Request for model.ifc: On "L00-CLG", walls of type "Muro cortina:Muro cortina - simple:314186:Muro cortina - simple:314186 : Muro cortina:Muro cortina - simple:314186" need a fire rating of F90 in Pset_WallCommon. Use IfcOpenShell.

First a look at what the model holds.

```python
import ifcopenshell
import ifcopenshell.util.element

model = ifcopenshell.open("model.ifc")
print(model.schema)
storey = next(s for s in model.by_type("IfcBuildingStorey") if s.Name == "L00-CLG")
walls = [e for e in ifcopenshell.util.element.get_decomposition(storey) if e.is_a("IfcWall")]
seen = {}
for e in walls:
    element_type = ifcopenshell.util.element.get_type(e)
    key = (element_type.Name if element_type != e and element_type else None, ifcopenshell.util.element.get_pset(e, "Pset_WallCommon", "FireRating"))
    seen[key] = seen.get(key, 0) + 1
for (name, value), count in sorted(seen.items(), key=str):
    print(count, "x", name, "|", value)
```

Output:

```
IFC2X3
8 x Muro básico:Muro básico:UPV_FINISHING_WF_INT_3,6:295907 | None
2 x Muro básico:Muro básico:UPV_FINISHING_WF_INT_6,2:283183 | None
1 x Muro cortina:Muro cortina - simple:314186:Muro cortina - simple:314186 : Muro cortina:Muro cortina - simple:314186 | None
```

```python
import ifcopenshell
import ifcopenshell.api.pset
import ifcopenshell.util.element

model = ifcopenshell.open("model.ifc")

storey = next(s for s in model.by_type("IfcBuildingStorey") if s.Name == "L00-CLG")
walls = [e for e in ifcopenshell.util.element.get_decomposition(storey) if e.is_a("IfcWall")]

count = 0
for e in walls:
    element_type = ifcopenshell.util.element.get_type(e)
    if element_type in (None, e) or element_type.Name != "Muro cortina:Muro cortina - simple:314186:Muro cortina - simple:314186 : Muro cortina:Muro cortina - simple:314186":
        continue
    # add_pset returns the element's existing set when there is one.
    pset = ifcopenshell.api.pset.add_pset(model, product=e, name="Pset_WallCommon")
    ifcopenshell.api.pset.edit_pset(model, pset=pset, properties={"FireRating": "F90"})
    count += 1

print(count, "walls updated")

model.write("model_updated.ifc")
```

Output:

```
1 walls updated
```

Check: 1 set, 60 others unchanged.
